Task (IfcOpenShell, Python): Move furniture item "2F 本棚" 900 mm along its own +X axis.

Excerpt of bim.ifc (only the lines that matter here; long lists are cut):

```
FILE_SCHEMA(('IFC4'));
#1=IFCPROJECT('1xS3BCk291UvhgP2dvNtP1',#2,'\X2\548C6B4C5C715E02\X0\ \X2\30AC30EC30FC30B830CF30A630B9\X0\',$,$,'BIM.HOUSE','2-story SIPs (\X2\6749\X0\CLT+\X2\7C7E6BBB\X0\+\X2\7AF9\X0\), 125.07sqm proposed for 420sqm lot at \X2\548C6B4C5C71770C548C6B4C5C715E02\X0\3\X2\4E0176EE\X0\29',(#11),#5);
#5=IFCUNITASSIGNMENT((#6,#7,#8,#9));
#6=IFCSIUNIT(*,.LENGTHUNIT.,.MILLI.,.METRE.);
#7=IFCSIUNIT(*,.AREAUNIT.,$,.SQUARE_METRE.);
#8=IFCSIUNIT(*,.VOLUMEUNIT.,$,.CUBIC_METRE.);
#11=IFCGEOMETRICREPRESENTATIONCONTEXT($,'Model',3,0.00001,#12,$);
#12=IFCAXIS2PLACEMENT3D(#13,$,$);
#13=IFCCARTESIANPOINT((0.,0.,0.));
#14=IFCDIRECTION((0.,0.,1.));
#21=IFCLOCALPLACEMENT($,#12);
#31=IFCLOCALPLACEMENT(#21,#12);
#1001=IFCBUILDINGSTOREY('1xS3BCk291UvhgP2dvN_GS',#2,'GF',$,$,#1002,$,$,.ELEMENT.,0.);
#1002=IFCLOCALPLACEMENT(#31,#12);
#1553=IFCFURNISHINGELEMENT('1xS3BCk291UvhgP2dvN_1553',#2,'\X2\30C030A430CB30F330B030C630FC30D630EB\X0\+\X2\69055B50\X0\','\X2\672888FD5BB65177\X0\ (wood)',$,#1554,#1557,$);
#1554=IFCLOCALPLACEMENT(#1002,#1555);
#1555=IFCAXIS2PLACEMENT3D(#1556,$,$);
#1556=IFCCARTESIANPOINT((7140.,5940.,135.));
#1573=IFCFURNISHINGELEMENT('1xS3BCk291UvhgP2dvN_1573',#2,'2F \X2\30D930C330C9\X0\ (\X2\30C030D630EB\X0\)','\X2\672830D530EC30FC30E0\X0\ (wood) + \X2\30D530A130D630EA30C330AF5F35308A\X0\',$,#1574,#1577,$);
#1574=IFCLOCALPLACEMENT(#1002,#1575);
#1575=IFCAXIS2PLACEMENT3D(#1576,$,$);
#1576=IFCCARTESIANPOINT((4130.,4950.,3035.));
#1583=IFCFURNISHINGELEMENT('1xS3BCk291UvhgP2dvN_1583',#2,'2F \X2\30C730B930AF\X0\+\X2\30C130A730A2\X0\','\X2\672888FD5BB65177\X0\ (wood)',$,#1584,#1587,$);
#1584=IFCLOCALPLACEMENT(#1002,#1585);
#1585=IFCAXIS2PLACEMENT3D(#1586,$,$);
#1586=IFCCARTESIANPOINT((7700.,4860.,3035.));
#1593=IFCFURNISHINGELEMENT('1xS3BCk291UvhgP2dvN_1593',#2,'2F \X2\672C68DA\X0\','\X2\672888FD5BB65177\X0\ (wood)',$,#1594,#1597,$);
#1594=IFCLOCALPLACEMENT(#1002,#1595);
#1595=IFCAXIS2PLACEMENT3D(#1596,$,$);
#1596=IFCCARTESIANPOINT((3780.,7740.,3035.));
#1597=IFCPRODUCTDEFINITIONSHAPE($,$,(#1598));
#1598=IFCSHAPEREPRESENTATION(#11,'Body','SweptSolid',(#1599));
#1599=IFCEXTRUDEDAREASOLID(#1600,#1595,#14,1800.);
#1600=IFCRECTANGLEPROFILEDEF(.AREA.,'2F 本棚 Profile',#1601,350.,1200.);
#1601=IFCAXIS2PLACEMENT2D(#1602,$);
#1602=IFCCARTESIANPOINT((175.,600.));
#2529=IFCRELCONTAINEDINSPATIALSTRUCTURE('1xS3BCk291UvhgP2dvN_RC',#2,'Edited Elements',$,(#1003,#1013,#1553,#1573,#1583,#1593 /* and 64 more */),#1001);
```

```python
import ifcopenshell
import ifcopenshell.api.geometry
import ifcopenshell.util.placement
import ifcopenshell.util.unit

model = ifcopenshell.open("bim.ifc")
unit_scale = ifcopenshell.util.unit.calculate_unit_scale(model)

item = model.by_guid("1xS3BCk291UvhgP2dvN_1593")
matrix = ifcopenshell.util.placement.get_local_placement(item.ObjectPlacement)
matrix[:3, 3] += matrix[:3, 0] * 0.9 / unit_scale
ifcopenshell.api.geometry.edit_object_placement(model, product=item, matrix=matrix, is_si=False)

print(ifcopenshell.util.placement.get_local_placement(item.ObjectPlacement).round(3) + 0.0)

model.write("bim_edited.ifc")
```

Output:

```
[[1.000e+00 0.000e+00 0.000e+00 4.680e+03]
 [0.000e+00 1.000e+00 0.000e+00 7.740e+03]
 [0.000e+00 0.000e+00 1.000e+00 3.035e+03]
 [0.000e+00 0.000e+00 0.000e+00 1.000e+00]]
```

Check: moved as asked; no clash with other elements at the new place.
